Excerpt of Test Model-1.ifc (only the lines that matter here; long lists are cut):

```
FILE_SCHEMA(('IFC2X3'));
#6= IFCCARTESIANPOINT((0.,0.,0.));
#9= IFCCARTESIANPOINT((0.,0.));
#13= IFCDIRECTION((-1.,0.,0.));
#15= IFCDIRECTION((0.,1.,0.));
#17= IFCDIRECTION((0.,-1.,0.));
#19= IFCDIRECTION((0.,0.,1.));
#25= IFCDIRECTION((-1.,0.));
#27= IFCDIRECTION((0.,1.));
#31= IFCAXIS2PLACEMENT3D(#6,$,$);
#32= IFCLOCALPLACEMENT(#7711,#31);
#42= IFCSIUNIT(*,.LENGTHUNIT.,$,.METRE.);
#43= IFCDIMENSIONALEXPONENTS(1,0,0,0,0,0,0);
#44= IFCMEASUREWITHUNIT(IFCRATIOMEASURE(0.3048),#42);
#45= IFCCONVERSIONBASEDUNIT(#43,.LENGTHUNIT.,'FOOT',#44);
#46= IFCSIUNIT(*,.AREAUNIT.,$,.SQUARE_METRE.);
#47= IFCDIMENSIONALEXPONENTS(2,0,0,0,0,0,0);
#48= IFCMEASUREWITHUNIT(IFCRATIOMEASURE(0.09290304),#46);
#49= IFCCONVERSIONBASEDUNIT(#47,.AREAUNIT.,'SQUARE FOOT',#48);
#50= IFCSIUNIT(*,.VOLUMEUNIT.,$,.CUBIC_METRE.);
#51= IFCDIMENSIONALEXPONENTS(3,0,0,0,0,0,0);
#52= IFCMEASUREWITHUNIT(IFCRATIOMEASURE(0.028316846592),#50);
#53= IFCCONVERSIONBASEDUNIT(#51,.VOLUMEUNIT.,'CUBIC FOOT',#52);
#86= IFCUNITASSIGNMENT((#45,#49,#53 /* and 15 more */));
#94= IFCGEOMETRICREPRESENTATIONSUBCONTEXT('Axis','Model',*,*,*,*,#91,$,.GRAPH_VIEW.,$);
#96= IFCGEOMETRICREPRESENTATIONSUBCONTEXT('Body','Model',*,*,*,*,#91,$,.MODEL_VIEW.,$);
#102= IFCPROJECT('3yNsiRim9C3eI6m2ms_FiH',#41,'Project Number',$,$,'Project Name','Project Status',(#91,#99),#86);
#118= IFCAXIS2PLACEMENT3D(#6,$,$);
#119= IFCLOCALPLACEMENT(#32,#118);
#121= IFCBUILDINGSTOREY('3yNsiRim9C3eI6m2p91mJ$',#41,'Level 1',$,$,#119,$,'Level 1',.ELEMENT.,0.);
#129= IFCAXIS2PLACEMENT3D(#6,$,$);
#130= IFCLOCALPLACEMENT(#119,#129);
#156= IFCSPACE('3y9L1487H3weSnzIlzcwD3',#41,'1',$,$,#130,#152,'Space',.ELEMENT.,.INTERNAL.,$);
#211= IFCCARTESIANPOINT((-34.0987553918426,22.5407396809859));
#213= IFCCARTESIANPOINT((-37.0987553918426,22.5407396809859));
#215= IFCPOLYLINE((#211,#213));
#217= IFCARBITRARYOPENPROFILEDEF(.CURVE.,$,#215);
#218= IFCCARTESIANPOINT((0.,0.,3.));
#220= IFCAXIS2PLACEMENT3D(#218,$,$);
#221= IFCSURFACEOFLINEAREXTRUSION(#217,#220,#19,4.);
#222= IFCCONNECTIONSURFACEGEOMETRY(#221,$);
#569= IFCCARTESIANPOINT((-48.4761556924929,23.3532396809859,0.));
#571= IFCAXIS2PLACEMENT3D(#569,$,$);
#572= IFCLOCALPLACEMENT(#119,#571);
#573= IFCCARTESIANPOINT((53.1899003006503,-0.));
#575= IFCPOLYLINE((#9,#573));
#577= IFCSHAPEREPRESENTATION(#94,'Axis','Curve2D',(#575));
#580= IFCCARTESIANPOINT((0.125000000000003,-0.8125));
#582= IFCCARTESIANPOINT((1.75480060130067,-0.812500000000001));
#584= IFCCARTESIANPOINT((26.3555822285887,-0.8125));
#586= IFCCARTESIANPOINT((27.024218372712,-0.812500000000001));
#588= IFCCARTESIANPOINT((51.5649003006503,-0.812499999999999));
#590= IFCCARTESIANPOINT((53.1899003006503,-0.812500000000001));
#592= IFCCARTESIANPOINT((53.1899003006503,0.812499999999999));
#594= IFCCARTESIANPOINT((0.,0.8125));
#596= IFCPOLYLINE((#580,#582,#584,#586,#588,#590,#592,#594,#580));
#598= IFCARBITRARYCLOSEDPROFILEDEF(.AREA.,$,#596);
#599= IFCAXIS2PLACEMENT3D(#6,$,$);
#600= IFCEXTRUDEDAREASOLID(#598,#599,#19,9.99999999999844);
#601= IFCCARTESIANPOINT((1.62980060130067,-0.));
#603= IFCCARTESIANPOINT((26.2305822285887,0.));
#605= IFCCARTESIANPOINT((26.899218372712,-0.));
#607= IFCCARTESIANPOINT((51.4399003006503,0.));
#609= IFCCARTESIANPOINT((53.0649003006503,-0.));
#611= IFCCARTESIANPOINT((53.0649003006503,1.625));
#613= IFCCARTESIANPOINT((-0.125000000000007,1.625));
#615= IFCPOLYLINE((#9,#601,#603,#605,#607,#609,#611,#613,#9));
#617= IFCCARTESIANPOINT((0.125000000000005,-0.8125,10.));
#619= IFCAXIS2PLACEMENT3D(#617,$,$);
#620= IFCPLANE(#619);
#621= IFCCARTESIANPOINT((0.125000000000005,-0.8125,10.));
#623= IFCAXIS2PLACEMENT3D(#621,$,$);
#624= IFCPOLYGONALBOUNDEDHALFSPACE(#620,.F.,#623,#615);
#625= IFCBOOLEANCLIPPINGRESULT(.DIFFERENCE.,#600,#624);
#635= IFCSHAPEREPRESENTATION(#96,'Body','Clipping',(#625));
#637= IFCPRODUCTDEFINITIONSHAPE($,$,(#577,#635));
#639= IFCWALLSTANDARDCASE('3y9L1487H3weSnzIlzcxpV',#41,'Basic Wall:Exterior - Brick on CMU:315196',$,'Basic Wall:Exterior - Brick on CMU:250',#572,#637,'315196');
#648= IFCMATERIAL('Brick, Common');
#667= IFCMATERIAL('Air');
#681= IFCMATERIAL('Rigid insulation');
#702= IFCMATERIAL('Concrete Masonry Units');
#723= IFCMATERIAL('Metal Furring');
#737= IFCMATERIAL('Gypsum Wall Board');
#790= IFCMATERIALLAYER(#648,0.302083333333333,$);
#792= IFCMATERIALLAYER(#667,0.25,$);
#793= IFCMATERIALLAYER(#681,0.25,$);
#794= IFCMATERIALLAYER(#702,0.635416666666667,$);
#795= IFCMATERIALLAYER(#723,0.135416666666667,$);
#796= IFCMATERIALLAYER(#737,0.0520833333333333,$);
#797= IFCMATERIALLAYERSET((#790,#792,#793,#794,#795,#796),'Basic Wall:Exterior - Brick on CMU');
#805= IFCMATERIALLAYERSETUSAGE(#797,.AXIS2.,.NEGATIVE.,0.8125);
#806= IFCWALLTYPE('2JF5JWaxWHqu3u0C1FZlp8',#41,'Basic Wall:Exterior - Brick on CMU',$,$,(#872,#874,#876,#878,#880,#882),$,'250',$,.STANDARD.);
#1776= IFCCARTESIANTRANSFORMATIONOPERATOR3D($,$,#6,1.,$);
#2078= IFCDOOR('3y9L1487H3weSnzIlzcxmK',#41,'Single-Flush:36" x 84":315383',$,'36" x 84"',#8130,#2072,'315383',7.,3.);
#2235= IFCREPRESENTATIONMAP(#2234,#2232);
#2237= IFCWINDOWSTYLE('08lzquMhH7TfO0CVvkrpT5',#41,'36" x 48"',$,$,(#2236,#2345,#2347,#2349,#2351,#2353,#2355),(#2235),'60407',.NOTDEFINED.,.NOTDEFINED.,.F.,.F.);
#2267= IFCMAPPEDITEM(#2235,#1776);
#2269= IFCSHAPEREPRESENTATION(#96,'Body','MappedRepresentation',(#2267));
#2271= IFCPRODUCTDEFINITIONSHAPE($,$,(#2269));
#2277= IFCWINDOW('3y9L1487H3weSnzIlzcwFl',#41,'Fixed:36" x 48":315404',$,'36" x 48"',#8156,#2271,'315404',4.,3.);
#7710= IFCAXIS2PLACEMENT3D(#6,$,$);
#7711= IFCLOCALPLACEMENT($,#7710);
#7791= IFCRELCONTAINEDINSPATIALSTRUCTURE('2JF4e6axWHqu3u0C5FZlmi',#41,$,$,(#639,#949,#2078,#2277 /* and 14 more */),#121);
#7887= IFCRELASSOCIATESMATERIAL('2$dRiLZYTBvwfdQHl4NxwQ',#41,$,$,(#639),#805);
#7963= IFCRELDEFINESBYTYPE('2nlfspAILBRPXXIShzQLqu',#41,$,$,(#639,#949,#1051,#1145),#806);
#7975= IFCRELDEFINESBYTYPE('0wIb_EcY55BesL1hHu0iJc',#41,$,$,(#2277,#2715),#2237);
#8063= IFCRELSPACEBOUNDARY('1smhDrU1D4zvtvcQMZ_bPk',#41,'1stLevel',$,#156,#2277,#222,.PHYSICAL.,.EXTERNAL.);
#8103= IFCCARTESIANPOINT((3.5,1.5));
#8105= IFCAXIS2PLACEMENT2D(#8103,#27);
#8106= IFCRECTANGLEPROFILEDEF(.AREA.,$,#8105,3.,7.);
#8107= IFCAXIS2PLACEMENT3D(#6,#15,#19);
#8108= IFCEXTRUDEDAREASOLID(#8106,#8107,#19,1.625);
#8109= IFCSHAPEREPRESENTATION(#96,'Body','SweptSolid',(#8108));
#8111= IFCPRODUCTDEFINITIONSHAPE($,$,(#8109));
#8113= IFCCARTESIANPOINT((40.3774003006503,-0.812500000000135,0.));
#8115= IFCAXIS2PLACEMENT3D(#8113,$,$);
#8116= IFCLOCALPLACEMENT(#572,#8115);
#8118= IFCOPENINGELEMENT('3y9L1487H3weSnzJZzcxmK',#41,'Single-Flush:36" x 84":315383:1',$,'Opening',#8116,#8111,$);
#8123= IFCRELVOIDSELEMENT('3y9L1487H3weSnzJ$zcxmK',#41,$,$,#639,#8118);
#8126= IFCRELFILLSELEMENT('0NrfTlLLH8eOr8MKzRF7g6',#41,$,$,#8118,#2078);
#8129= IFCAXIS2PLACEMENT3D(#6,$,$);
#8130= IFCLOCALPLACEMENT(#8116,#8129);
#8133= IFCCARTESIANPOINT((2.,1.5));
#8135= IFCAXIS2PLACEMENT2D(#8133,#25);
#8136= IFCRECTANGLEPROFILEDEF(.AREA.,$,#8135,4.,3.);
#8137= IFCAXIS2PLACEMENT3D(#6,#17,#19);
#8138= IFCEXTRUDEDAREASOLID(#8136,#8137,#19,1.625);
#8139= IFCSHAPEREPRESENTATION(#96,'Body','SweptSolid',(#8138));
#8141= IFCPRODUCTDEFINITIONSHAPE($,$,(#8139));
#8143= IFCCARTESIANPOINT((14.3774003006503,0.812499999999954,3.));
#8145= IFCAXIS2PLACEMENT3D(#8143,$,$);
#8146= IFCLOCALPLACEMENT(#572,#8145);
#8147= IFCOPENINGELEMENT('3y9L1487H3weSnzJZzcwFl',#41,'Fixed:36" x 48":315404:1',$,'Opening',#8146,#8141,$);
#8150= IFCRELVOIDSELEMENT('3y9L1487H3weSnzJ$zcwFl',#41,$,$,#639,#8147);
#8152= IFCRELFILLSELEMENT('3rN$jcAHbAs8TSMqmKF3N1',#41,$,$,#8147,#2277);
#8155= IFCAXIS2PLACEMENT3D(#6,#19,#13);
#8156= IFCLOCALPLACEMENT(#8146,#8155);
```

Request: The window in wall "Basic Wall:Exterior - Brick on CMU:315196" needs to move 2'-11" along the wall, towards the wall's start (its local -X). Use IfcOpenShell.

```python
import numpy as np
import ifcopenshell
import ifcopenshell.api.geometry
import ifcopenshell.util.placement
import ifcopenshell.util.unit

model = ifcopenshell.open("Test Model-1.ifc")
unit_scale = ifcopenshell.util.unit.calculate_unit_scale(model)

window = model.by_guid("3y9L1487H3weSnzIlzcwFl")
opening = window.FillsVoids[0].RelatingOpeningElement
wall = opening.VoidsElements[0].RelatingBuildingElement

wall_matrix = ifcopenshell.util.placement.get_local_placement(wall.ObjectPlacement)
shift = wall_matrix[:3, 0] * -35 * 0.0254 / unit_scale
before = ifcopenshell.util.placement.get_local_placement(window.ObjectPlacement)[:3, 3].copy()

# The window is placed relative to its opening, so it follows when the opening moves.
matrix = ifcopenshell.util.placement.get_local_placement(opening.ObjectPlacement)
matrix[:3, 3] += shift
ifcopenshell.api.geometry.edit_object_placement(
    model, product=opening, matrix=matrix, is_si=False, should_transform_children=True
)

# Space boundary surfaces are stored in each space's coordinates; move them too.
for rel in window.ProvidesBoundaries:
    if not rel.ConnectionGeometry:
        continue
    surface = rel.ConnectionGeometry.SurfaceOnRelatingElement
    space_matrix = ifcopenshell.util.placement.get_local_placement(rel.RelatingSpace.ObjectPlacement)
    point = np.array(surface.Position.Location.Coordinates) + space_matrix[:3, :3].T @ shift
    surface.Position = model.createIfcAxis2Placement3D(
        model.createIfcCartesianPoint(point.tolist()), surface.Position.Axis, surface.Position.RefDirection
    )

after = ifcopenshell.util.placement.get_local_placement(window.ObjectPlacement)[:3, 3]
print("window moved by", (after - before).round(3) + 0.0)

model.write("Test Model-1_edited.ifc")
```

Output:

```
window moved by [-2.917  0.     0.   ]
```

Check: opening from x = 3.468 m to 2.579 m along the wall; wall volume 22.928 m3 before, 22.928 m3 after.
